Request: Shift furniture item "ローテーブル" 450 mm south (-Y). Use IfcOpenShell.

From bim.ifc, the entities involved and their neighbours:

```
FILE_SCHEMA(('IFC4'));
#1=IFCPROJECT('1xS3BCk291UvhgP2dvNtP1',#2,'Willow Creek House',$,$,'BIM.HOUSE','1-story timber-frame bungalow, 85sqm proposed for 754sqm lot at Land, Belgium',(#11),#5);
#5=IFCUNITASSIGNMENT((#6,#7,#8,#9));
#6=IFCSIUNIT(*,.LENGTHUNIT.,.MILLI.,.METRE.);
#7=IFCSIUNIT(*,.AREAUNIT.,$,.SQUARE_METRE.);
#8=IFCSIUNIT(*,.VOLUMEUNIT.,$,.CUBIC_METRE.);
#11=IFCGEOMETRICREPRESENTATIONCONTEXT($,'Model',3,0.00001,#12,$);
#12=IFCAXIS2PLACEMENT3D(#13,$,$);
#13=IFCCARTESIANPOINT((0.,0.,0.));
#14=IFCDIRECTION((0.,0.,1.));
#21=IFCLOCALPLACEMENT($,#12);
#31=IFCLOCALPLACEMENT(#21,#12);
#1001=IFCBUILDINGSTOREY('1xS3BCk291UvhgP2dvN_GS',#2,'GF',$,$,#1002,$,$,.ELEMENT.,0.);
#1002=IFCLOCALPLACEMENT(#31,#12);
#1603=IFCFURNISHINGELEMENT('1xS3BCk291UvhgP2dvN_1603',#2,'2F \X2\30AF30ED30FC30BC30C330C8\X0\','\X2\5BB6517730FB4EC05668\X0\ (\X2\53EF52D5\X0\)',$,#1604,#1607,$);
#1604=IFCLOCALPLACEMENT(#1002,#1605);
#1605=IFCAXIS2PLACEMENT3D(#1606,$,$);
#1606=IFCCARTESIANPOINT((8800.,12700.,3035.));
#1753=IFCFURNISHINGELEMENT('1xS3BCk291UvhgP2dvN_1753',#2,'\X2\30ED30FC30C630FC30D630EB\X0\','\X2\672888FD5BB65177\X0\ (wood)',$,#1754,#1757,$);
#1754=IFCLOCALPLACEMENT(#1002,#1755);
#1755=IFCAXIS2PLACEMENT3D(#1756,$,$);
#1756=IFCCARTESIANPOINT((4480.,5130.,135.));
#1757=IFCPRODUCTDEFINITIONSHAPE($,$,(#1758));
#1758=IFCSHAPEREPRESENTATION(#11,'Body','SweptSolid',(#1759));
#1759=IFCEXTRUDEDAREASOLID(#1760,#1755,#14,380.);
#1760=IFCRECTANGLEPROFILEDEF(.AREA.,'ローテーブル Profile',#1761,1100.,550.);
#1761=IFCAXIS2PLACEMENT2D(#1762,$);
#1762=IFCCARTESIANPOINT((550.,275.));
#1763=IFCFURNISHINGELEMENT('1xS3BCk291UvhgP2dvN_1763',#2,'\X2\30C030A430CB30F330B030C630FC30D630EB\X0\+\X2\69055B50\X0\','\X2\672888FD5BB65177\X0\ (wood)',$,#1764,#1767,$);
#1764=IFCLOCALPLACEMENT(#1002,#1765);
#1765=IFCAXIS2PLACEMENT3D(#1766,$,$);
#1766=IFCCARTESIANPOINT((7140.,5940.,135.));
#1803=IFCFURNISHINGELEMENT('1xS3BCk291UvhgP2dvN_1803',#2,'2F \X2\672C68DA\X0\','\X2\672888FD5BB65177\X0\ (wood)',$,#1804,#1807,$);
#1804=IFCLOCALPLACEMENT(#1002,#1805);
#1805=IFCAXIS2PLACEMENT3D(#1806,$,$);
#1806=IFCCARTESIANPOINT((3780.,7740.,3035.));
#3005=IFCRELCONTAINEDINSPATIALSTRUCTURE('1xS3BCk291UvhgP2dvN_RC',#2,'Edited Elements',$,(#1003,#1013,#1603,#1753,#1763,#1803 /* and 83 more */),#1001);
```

```python
import ifcopenshell
import ifcopenshell.api.geometry
import ifcopenshell.util.placement

model = ifcopenshell.open("bim.ifc")

item = model.by_guid("1xS3BCk291UvhgP2dvN_1753")
matrix = ifcopenshell.util.placement.get_local_placement(item.ObjectPlacement)
matrix[1, 3] -= 450.0
ifcopenshell.api.geometry.edit_object_placement(model, product=item, matrix=matrix, is_si=False)

print(ifcopenshell.util.placement.get_local_placement(item.ObjectPlacement).round(3) + 0.0)

model.write("bim_edited.ifc")
```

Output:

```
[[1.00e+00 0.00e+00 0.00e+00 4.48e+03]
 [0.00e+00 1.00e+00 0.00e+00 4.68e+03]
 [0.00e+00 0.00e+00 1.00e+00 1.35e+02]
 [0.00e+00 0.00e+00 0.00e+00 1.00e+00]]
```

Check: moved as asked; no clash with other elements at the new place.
